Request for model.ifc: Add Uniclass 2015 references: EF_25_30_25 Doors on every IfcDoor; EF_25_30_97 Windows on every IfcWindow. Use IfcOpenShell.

First a look at what the model holds.

```python
import ifcopenshell

model = ifcopenshell.open("model.ifc")
print(model.schema)
print("classifications:", [c.Name for c in model.by_type("IfcClassification")])
for ifc_class in ("IfcDoor", "IfcRoof", "IfcStair", "IfcWall", "IfcWindow"):
    print(ifc_class, len(model.by_type(ifc_class)))
```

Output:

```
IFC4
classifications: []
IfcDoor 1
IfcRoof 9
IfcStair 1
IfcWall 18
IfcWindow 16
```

```python
import ifcopenshell
import ifcopenshell.api.classification

model = ifcopenshell.open("model.ifc")

system = ifcopenshell.api.classification.add_classification(model, classification="Uniclass 2015")

codes = {
    "IfcDoor": ("EF_25_30_25", "Doors"),
    "IfcWindow": ("EF_25_30_97", "Windows"),
}
for ifc_class, (code, name) in codes.items():
    products = model.by_type(ifc_class)
    ifcopenshell.api.classification.add_reference(
        model, products=products, classification=system, identification=code, name=name
    )
    print(code, len(products))

model.write("model-out.ifc")
```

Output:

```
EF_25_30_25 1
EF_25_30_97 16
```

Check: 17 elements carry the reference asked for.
